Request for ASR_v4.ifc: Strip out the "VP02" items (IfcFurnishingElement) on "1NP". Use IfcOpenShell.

First a look at what the model holds.

```python
import ifcopenshell
import ifcopenshell.util.element

model = ifcopenshell.open("ASR_v4.ifc")
print(model.schema)
storey = next(s for s in model.by_type("IfcBuildingStorey") if s.Name == "1NP")
furniture = [e for e in ifcopenshell.util.element.get_decomposition(storey) if e.is_a("IfcFurnishingElement")]
seen = {}
for e in furniture:
    element_type = ifcopenshell.util.element.get_type(e)
    name = element_type.Name if element_type not in (None, e) else None
    seen[name] = seen.get(name, 0) + 1
for name, count in sorted(seen.items(), key=str):
    print(count, "x", name)
```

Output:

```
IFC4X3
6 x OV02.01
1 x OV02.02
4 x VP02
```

```python
import ifcopenshell
import ifcopenshell.api.root
import ifcopenshell.util.element

model = ifcopenshell.open("ASR_v4.ifc")

storey = next(s for s in model.by_type("IfcBuildingStorey") if s.Name == "1NP")
furniture = [e for e in ifcopenshell.util.element.get_decomposition(storey) if e.is_a("IfcFurnishingElement")]
targets = [e for e in furniture if (t := ifcopenshell.util.element.get_type(e)) not in (None, e) and t.Name == "VP02"]

for e in targets:
    ifcopenshell.api.root.remove_product(model, product=e)
print(len(targets), "removed")

model.write("ASR_v4-out.ifc")
```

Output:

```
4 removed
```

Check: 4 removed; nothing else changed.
